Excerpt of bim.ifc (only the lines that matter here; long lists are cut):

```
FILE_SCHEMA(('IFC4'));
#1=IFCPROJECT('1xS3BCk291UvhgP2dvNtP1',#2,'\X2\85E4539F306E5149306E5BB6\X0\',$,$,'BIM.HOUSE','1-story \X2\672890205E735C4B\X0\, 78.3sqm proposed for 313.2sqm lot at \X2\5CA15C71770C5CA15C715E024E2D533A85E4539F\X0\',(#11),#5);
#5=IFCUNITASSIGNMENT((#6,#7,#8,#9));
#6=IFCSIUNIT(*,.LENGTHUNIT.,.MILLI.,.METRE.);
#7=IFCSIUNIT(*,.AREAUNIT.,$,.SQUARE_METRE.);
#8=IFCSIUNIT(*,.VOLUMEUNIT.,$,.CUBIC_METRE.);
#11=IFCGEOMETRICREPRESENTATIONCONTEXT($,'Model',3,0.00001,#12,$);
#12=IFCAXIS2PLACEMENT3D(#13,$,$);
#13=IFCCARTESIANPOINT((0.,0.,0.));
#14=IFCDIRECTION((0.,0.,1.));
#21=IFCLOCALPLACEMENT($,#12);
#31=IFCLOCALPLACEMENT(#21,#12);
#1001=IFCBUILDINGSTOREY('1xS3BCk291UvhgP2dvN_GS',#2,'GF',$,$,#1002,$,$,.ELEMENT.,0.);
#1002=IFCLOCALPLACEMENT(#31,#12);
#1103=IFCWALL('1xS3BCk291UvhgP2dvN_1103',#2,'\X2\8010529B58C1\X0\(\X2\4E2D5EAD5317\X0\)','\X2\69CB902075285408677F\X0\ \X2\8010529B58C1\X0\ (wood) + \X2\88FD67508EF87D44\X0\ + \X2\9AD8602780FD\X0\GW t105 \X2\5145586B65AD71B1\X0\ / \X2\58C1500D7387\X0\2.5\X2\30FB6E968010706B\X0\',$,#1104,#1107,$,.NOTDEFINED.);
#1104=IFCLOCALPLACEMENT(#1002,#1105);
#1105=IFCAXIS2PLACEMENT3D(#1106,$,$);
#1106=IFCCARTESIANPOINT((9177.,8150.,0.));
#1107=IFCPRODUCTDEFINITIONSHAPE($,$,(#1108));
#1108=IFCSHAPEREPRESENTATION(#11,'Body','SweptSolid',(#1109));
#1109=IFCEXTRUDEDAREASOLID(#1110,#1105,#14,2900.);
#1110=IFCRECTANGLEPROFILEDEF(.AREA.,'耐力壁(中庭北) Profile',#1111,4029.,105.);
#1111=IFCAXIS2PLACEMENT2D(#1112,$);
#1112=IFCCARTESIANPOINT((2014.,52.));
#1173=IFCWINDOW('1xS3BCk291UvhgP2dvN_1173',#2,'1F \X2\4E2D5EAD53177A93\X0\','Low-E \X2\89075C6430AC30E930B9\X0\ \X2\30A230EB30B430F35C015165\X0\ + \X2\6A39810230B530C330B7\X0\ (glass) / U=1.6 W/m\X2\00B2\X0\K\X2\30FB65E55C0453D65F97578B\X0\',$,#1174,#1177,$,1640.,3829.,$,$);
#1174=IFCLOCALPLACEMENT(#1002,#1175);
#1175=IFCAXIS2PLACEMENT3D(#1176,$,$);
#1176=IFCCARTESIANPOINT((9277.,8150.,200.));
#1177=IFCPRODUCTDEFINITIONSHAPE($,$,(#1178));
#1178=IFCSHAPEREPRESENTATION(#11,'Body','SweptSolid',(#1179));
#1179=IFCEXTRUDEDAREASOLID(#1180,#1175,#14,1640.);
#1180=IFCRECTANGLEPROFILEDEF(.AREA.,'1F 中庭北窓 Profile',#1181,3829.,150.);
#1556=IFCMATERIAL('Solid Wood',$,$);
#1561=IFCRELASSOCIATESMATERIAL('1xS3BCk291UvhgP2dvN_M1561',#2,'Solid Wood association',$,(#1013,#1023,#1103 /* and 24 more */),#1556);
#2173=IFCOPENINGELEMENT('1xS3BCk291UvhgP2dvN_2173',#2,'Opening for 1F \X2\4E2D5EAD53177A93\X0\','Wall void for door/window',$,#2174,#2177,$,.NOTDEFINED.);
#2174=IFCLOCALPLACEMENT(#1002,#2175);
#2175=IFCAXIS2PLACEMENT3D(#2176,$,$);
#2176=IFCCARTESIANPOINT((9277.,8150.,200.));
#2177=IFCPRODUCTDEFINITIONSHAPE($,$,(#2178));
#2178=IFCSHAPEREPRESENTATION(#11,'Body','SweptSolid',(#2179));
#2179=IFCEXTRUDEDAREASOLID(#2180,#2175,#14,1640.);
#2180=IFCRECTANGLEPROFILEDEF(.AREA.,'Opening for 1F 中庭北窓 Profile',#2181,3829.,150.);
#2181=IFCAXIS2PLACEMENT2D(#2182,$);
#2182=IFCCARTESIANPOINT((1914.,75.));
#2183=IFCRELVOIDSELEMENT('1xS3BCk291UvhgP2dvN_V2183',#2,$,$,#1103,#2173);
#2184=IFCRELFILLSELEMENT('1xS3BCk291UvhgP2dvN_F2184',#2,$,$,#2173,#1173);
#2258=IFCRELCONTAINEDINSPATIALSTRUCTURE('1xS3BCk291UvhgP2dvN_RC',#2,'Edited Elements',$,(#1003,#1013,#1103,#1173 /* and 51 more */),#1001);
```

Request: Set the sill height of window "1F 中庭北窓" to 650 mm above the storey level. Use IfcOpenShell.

```python
import numpy as np
import ifcopenshell
import ifcopenshell.api.geometry
import ifcopenshell.geom
import ifcopenshell.util.element
import ifcopenshell.util.placement
import ifcopenshell.util.shape
import ifcopenshell.util.unit

model = ifcopenshell.open("bim.ifc")
unit_scale = ifcopenshell.util.unit.calculate_unit_scale(model)

window = model.by_guid("1xS3BCk291UvhgP2dvN_1173")
opening = window.FillsVoids[0].RelatingOpeningElement
storey = ifcopenshell.util.element.get_container(window, ifc_class="IfcBuildingStorey")
level = ifcopenshell.util.placement.get_local_placement(storey.ObjectPlacement)[2, 3]

# The opening's origin need not be at the sill, so measure its lowest point.
shape = ifcopenshell.geom.create_shape(ifcopenshell.geom.settings(), opening)
bottom = ifcopenshell.util.shape.get_shape_bottom_elevation(shape, shape.geometry) / unit_scale
dz = level + 0.65 / unit_scale - bottom

shift = np.array([0.0, 0.0, dz])
# The window is not placed relative to its opening, so move both.
for product in (opening, window):
    matrix = ifcopenshell.util.placement.get_local_placement(product.ObjectPlacement)
    matrix[:3, 3] += shift
    ifcopenshell.api.geometry.edit_object_placement(model, product=product, matrix=matrix, is_si=False)

print(f"moved by {dz * unit_scale:+.3f} m")

model.write("bim_updated.ifc")
```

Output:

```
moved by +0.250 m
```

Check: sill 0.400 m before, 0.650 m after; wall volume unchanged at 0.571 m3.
